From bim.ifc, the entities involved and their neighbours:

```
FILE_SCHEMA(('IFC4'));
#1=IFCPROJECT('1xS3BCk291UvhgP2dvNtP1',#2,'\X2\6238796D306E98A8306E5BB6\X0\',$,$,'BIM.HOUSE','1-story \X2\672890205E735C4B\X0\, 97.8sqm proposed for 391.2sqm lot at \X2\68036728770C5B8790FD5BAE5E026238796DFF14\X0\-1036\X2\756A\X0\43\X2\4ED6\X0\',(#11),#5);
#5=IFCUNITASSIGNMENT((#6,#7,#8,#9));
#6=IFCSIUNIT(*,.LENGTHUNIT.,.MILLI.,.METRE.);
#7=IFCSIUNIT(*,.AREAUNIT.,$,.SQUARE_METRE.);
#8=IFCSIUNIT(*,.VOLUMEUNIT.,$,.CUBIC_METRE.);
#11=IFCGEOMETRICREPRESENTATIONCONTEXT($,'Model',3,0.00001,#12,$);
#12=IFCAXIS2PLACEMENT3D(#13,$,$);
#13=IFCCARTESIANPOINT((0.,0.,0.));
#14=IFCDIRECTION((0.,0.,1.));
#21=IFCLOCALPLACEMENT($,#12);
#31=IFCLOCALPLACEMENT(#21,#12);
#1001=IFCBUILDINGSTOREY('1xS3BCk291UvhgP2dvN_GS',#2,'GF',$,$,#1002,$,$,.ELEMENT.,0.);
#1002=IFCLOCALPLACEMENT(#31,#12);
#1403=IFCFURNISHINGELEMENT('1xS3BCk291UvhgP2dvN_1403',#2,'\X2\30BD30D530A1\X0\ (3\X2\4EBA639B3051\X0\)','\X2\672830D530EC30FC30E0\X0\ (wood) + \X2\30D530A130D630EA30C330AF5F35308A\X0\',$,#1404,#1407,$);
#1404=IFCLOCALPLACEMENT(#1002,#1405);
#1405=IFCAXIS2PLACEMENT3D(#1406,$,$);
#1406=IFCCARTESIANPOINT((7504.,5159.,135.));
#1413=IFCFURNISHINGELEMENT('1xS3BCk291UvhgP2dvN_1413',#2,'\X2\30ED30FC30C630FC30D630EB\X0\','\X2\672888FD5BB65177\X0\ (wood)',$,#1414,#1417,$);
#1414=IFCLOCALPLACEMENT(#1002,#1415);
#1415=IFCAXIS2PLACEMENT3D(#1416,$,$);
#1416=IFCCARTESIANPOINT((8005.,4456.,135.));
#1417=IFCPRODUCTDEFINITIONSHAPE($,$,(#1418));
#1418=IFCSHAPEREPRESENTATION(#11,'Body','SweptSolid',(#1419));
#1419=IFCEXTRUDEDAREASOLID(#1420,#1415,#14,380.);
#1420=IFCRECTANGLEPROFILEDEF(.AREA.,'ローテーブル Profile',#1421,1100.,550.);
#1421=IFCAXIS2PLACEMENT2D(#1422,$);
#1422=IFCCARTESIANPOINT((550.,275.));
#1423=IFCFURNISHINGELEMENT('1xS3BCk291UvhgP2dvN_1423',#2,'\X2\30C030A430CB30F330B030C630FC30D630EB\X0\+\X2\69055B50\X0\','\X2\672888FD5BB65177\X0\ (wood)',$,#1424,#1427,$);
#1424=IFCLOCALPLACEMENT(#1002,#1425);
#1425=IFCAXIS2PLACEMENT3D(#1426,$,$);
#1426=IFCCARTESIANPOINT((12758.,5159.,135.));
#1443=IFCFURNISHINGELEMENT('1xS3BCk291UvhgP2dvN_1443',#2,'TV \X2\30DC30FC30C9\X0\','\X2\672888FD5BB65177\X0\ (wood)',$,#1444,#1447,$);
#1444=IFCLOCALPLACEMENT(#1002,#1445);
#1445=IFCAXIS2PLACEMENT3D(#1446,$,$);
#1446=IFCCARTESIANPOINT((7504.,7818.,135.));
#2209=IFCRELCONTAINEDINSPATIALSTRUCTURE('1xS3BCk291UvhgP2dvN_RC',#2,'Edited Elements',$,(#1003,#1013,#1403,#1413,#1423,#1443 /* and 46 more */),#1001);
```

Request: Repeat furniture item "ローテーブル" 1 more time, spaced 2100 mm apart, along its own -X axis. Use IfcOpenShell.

```python
import ifcopenshell
import ifcopenshell.api.geometry
import ifcopenshell.api.root
import ifcopenshell.util.element
import ifcopenshell.util.placement

model = ifcopenshell.open("bim.ifc")


def reuse_history(source, copy):
    """copy_class also copies each property set's owner history, people and application; keep the originals."""
    for rel in copy.IsDefinedBy:
        if rel.is_a("IfcRelDefinesByProperties") and (history := rel.RelatingPropertyDefinition.OwnerHistory):
            rel.RelatingPropertyDefinition.OwnerHistory = source.OwnerHistory
            ifcopenshell.util.element.remove_deep2(model, history)


source = model.by_guid("1xS3BCk291UvhgP2dvN_1413")
base = ifcopenshell.util.placement.get_local_placement(source.ObjectPlacement)
step = -base[:3, 0] * 2100.0

for i in range(1, 2):
    copy = ifcopenshell.api.root.copy_class(model, product=source)
    copy.Representation = ifcopenshell.util.element.copy_deep(
        model, source.Representation, exclude=["IfcGeometricRepresentationContext", "IfcRepresentationMap"]
    )
    reuse_history(source, copy)
    matrix = base.copy()
    matrix[:3, 3] += i * step
    print("added at", matrix[:3, 3].round(3) + 0.0)
    ifcopenshell.api.geometry.edit_object_placement(model, product=copy, matrix=matrix, is_si=False)

model.write("bim_v2.ifc")
```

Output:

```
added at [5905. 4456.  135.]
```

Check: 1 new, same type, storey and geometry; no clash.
